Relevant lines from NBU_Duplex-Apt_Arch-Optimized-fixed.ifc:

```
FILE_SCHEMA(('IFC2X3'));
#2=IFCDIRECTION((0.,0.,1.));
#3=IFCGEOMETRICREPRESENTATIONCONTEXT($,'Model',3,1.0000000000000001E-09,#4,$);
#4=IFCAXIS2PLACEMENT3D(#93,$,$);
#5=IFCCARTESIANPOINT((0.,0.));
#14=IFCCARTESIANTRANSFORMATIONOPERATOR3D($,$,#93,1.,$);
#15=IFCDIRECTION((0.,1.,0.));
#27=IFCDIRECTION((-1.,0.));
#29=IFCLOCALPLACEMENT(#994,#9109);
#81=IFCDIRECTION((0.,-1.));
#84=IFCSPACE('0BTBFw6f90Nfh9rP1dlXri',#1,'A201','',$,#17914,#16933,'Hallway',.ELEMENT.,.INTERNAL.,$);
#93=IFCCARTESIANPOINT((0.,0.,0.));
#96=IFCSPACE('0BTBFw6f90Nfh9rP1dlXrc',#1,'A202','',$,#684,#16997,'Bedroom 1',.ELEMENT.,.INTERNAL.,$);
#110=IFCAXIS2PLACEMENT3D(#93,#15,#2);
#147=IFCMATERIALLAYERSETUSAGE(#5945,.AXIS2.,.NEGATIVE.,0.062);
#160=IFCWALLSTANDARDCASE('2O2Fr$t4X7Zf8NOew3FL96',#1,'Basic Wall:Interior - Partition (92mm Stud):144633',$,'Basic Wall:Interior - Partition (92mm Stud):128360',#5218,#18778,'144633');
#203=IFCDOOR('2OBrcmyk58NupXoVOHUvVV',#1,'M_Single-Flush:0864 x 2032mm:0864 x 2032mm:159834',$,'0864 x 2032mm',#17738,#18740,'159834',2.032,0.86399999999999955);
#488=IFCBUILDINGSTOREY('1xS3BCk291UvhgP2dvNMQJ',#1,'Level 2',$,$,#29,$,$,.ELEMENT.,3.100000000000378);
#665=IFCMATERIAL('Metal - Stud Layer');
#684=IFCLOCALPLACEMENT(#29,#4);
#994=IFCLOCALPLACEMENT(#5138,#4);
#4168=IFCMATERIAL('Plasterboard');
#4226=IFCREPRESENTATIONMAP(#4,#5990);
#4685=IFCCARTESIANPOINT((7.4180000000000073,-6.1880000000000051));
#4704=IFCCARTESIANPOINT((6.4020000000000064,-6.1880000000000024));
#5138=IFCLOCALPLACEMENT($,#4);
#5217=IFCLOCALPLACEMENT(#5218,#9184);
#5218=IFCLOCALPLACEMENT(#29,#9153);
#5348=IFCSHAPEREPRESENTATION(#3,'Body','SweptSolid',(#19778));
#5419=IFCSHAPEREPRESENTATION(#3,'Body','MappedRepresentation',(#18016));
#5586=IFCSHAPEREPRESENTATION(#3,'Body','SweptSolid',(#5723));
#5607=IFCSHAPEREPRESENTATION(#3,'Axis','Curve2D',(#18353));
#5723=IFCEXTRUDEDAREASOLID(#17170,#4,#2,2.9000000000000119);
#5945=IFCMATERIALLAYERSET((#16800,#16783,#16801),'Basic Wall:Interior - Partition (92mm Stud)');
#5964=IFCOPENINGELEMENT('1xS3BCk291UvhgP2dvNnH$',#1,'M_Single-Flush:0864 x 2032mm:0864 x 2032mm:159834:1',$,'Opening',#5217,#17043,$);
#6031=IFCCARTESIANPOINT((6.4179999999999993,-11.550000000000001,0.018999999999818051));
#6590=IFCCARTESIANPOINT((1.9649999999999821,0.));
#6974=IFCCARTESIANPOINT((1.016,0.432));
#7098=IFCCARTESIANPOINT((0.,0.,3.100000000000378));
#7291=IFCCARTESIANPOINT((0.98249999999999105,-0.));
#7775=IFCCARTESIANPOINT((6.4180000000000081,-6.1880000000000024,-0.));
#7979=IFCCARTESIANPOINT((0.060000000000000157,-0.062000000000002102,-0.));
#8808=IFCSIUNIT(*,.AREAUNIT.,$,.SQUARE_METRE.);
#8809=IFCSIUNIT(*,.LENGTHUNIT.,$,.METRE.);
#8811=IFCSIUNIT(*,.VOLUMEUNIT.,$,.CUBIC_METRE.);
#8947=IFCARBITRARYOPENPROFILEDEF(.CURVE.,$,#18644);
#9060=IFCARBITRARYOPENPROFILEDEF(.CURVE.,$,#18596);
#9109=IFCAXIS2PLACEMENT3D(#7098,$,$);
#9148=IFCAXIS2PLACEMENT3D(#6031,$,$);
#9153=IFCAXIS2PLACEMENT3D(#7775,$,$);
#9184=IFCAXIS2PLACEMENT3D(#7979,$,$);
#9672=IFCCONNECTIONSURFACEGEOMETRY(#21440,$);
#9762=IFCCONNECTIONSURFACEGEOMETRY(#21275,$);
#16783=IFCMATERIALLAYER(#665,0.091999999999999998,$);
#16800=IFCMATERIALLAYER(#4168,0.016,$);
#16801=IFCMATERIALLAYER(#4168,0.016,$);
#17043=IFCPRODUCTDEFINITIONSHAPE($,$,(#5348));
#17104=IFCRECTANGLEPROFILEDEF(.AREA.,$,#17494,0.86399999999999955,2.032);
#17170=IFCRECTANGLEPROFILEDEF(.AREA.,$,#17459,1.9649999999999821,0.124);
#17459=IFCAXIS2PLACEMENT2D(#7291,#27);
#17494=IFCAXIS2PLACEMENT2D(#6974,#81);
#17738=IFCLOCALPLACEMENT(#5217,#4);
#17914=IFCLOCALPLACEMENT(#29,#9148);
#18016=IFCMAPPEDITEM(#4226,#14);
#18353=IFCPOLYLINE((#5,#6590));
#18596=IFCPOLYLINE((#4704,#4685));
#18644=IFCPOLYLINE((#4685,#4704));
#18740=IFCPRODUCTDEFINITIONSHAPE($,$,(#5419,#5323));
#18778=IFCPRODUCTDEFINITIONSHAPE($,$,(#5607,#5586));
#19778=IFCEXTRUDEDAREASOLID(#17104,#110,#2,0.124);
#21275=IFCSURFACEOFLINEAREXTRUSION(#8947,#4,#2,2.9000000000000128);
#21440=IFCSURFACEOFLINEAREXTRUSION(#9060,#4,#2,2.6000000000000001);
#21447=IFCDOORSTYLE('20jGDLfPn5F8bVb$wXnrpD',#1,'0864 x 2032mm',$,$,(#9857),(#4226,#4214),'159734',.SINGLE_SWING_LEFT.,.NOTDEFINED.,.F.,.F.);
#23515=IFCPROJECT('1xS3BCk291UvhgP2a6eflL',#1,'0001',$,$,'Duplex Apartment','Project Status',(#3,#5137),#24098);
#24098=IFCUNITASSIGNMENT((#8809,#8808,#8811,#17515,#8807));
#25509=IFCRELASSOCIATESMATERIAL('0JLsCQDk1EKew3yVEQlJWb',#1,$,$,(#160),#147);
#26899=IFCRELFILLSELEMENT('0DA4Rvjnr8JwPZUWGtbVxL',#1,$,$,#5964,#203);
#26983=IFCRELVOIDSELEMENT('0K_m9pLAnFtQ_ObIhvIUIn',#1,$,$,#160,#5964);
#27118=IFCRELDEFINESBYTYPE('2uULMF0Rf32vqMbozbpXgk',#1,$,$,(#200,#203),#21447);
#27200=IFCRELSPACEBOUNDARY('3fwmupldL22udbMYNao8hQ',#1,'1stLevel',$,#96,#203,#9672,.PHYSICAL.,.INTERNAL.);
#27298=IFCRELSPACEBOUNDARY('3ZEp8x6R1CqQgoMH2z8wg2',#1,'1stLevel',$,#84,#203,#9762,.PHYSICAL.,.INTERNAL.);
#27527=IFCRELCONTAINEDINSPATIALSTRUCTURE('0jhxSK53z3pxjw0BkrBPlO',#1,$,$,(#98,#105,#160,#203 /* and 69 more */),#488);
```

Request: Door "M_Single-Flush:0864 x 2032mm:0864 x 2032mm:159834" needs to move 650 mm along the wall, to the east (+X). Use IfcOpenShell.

```python
import numpy as np
import ifcopenshell
import ifcopenshell.api.geometry
import ifcopenshell.util.placement
import ifcopenshell.util.unit

model = ifcopenshell.open("NBU_Duplex-Apt_Arch-Optimized-fixed.ifc")
unit_scale = ifcopenshell.util.unit.calculate_unit_scale(model)

door = model.by_guid("2OBrcmyk58NupXoVOHUvVV")
opening = door.FillsVoids[0].RelatingOpeningElement
wall = opening.VoidsElements[0].RelatingBuildingElement

wall_matrix = ifcopenshell.util.placement.get_local_placement(wall.ObjectPlacement)
shift = wall_matrix[:3, 0] * 0.65 / unit_scale
before = ifcopenshell.util.placement.get_local_placement(door.ObjectPlacement)[:3, 3].copy()

# The door is placed relative to its opening, so it follows when the opening moves.
matrix = ifcopenshell.util.placement.get_local_placement(opening.ObjectPlacement)
matrix[:3, 3] += shift
ifcopenshell.api.geometry.edit_object_placement(
    model, product=opening, matrix=matrix, is_si=False, should_transform_children=True
)

# Space boundary surfaces are stored in each space's coordinates; move them too.
for rel in door.ProvidesBoundaries:
    if not rel.ConnectionGeometry:
        continue
    surface = rel.ConnectionGeometry.SurfaceOnRelatingElement
    space_matrix = ifcopenshell.util.placement.get_local_placement(rel.RelatingSpace.ObjectPlacement)
    point = np.array(surface.Position.Location.Coordinates) + space_matrix[:3, :3].T @ shift
    surface.Position = model.createIfcAxis2Placement3D(
        model.createIfcCartesianPoint(point.tolist()), surface.Position.Axis, surface.Position.RefDirection
    )

after = ifcopenshell.util.placement.get_local_placement(door.ObjectPlacement)[:3, 3]
print("door moved by", (after - before).round(3) + 0.0)

model.write("NBU_Duplex-Apt_Arch-Optimized-fixed_updated.ifc")
```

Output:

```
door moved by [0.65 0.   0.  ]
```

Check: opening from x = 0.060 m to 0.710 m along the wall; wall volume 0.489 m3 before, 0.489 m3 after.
